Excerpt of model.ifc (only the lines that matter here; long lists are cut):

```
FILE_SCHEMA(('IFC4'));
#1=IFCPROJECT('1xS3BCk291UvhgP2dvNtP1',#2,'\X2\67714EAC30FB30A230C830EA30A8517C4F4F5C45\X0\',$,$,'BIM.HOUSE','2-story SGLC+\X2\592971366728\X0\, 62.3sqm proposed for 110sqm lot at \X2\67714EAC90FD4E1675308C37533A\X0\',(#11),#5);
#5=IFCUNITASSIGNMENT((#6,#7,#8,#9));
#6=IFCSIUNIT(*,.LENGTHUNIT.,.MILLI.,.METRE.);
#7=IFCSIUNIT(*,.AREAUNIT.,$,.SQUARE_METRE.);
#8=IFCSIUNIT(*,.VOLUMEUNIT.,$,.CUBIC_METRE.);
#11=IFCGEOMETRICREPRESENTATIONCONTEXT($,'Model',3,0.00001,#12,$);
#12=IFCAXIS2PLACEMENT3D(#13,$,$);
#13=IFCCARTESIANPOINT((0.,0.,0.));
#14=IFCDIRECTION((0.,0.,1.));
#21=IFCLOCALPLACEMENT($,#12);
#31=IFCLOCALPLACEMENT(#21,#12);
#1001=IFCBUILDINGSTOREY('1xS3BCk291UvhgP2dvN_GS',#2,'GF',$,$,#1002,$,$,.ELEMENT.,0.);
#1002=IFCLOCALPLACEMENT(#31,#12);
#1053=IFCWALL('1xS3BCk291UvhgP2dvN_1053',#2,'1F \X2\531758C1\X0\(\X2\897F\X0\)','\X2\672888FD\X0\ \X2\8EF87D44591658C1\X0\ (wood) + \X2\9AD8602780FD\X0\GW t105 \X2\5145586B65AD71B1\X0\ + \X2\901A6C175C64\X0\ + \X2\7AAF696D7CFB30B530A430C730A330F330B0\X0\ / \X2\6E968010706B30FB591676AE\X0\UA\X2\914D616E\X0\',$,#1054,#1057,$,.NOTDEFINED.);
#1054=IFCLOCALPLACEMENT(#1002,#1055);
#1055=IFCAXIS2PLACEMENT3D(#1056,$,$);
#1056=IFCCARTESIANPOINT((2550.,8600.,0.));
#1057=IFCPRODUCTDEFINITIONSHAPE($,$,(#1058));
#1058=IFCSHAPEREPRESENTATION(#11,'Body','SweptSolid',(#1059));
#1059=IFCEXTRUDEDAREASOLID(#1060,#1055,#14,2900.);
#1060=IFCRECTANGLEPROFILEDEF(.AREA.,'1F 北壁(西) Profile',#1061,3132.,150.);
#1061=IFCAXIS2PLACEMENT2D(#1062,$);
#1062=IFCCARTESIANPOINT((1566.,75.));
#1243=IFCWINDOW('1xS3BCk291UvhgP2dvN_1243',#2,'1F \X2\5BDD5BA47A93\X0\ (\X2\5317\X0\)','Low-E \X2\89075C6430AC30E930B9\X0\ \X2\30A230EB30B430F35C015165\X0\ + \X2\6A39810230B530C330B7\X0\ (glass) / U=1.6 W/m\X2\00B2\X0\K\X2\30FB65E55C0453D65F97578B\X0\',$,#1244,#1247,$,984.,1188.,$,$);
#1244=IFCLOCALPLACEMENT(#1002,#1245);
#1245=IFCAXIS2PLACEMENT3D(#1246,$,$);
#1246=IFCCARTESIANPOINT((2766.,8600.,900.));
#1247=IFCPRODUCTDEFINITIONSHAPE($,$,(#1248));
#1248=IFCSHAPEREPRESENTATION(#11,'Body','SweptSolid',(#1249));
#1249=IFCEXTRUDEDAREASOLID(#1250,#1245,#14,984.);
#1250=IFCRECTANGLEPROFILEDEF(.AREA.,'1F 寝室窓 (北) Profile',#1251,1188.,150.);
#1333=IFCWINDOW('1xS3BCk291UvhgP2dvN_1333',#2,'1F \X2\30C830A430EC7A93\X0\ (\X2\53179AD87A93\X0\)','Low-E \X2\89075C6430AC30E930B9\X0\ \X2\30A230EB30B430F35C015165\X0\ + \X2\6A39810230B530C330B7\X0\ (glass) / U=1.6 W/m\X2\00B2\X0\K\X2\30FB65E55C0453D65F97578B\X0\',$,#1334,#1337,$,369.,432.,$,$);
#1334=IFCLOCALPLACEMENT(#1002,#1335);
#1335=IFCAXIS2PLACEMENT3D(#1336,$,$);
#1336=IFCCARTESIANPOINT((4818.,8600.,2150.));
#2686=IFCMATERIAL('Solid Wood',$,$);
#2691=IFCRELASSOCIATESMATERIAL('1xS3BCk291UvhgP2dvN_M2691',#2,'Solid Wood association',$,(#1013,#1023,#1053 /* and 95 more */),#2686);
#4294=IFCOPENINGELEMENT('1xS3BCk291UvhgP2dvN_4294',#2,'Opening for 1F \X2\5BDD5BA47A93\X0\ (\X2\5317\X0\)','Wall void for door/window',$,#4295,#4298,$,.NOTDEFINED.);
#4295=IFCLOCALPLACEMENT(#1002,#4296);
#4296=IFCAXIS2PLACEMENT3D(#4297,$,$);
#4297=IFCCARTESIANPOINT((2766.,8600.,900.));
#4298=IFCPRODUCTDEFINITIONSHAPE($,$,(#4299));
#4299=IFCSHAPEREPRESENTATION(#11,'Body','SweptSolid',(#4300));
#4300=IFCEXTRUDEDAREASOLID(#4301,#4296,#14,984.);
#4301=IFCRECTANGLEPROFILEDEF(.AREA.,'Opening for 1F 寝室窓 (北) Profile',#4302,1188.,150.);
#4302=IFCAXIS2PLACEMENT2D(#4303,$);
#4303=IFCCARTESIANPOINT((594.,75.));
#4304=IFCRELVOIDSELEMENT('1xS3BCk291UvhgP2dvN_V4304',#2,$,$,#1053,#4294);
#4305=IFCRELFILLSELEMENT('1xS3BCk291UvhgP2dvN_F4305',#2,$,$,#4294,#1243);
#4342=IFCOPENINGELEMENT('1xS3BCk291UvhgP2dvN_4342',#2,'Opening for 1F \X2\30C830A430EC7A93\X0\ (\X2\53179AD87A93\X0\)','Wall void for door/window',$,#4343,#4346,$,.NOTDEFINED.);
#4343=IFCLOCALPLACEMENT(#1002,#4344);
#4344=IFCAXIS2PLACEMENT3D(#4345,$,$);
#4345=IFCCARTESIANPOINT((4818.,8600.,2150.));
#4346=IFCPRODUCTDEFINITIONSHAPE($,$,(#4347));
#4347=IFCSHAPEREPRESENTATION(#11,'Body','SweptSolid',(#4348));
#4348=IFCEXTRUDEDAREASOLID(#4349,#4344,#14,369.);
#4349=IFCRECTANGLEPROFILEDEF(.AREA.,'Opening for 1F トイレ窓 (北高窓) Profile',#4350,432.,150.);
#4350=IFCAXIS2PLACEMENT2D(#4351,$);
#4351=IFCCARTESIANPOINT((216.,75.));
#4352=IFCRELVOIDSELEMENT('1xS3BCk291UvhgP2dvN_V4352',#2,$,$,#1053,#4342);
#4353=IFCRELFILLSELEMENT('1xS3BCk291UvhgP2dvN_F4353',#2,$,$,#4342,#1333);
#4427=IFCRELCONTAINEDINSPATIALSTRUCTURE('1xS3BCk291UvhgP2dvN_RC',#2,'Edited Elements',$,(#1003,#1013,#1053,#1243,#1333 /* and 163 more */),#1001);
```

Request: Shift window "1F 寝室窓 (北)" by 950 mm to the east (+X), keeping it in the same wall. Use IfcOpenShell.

```python
import ifcopenshell
import ifcopenshell.api.geometry
import ifcopenshell.util.placement
import ifcopenshell.util.unit

model = ifcopenshell.open("model.ifc")
unit_scale = ifcopenshell.util.unit.calculate_unit_scale(model)

window = model.by_id(1243)
opening = window.FillsVoids[0].RelatingOpeningElement
wall = opening.VoidsElements[0].RelatingBuildingElement

wall_matrix = ifcopenshell.util.placement.get_local_placement(wall.ObjectPlacement)
shift = wall_matrix[:3, 0] * 0.95 / unit_scale
before = ifcopenshell.util.placement.get_local_placement(window.ObjectPlacement)[:3, 3].copy()

# The window is not placed relative to its opening, so move both.
for product in (opening, window):
    matrix = ifcopenshell.util.placement.get_local_placement(product.ObjectPlacement)
    matrix[:3, 3] += shift
    ifcopenshell.api.geometry.edit_object_placement(model, product=product, matrix=matrix, is_si=False)

after = ifcopenshell.util.placement.get_local_placement(window.ObjectPlacement)[:3, 3]
print("window moved by", (after - before).round(3) + 0.0)

model.write("model-out.ifc")
```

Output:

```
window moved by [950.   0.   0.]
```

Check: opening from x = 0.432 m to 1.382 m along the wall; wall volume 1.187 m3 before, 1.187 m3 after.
